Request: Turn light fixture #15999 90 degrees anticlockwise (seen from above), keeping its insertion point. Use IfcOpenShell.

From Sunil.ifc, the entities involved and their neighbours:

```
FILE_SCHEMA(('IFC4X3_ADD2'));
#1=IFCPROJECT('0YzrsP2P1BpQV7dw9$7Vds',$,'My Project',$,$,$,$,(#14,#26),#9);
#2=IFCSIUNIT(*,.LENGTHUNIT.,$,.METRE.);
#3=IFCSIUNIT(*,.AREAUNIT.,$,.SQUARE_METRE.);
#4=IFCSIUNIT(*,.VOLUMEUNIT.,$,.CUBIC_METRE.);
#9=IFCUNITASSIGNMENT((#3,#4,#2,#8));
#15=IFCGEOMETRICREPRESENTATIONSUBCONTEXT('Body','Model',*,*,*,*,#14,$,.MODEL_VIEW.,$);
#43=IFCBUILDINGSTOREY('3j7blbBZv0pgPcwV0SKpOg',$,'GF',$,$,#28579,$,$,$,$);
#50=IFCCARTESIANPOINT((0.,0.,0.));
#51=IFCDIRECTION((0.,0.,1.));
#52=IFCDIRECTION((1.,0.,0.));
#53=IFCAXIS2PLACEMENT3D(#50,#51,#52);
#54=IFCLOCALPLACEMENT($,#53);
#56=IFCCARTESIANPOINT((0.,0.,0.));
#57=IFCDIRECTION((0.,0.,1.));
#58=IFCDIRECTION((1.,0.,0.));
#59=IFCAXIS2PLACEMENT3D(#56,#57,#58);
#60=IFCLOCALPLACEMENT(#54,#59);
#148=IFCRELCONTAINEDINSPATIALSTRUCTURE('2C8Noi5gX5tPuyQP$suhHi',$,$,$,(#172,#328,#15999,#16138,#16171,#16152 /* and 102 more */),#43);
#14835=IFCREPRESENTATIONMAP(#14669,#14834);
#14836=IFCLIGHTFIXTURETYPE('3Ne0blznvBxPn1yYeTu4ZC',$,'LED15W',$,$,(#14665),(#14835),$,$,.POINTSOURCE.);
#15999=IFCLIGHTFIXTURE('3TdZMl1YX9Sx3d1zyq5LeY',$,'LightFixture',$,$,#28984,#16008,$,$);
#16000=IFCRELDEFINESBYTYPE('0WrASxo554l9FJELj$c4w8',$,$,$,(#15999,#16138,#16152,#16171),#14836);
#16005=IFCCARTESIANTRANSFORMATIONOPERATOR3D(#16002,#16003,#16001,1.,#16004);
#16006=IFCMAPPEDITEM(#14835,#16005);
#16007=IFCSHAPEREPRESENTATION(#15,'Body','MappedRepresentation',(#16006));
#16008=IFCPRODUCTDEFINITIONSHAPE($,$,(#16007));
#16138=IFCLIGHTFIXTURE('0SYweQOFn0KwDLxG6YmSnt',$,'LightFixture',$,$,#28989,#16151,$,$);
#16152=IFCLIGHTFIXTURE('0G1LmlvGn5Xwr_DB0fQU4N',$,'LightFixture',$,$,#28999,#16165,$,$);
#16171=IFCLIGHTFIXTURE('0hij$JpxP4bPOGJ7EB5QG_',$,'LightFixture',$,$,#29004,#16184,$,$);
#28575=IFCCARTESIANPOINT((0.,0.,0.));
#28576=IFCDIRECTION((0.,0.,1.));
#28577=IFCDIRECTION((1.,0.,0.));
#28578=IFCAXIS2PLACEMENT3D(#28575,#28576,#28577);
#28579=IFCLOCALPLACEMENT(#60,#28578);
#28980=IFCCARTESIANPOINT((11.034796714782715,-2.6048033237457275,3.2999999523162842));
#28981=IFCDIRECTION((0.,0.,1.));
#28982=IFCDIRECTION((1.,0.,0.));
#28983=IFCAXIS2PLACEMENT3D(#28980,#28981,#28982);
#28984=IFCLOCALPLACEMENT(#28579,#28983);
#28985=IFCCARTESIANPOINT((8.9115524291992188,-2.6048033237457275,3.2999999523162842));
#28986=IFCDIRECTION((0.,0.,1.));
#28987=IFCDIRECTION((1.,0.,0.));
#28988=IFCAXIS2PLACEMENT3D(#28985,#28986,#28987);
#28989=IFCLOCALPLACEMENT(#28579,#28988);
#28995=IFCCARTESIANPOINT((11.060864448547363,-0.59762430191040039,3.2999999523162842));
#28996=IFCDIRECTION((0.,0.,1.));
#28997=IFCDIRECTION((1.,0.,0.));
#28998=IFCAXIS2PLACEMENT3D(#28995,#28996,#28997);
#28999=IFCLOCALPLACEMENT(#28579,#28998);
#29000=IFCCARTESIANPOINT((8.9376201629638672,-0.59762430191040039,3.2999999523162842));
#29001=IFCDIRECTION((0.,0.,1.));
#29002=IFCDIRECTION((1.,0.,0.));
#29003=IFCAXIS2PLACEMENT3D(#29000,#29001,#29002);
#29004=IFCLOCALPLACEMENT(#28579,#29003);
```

```python
import ifcopenshell
import ifcopenshell.api.geometry
import ifcopenshell.util.placement

model = ifcopenshell.open("Sunil.ifc")

item = model.by_guid("3TdZMl1YX9Sx3d1zyq5LeY")
matrix = ifcopenshell.util.placement.get_local_placement(item.ObjectPlacement)
matrix = matrix @ ifcopenshell.util.placement.rotation(90, "Z")
ifcopenshell.api.geometry.edit_object_placement(model, product=item, matrix=matrix, is_si=False)

print(ifcopenshell.util.placement.get_local_placement(item.ObjectPlacement).round(3) + 0.0)

model.write("Sunil_v2.ifc")
```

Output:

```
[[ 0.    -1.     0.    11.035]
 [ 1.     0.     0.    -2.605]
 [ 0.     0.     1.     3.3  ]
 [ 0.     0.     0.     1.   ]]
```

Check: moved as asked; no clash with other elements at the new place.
